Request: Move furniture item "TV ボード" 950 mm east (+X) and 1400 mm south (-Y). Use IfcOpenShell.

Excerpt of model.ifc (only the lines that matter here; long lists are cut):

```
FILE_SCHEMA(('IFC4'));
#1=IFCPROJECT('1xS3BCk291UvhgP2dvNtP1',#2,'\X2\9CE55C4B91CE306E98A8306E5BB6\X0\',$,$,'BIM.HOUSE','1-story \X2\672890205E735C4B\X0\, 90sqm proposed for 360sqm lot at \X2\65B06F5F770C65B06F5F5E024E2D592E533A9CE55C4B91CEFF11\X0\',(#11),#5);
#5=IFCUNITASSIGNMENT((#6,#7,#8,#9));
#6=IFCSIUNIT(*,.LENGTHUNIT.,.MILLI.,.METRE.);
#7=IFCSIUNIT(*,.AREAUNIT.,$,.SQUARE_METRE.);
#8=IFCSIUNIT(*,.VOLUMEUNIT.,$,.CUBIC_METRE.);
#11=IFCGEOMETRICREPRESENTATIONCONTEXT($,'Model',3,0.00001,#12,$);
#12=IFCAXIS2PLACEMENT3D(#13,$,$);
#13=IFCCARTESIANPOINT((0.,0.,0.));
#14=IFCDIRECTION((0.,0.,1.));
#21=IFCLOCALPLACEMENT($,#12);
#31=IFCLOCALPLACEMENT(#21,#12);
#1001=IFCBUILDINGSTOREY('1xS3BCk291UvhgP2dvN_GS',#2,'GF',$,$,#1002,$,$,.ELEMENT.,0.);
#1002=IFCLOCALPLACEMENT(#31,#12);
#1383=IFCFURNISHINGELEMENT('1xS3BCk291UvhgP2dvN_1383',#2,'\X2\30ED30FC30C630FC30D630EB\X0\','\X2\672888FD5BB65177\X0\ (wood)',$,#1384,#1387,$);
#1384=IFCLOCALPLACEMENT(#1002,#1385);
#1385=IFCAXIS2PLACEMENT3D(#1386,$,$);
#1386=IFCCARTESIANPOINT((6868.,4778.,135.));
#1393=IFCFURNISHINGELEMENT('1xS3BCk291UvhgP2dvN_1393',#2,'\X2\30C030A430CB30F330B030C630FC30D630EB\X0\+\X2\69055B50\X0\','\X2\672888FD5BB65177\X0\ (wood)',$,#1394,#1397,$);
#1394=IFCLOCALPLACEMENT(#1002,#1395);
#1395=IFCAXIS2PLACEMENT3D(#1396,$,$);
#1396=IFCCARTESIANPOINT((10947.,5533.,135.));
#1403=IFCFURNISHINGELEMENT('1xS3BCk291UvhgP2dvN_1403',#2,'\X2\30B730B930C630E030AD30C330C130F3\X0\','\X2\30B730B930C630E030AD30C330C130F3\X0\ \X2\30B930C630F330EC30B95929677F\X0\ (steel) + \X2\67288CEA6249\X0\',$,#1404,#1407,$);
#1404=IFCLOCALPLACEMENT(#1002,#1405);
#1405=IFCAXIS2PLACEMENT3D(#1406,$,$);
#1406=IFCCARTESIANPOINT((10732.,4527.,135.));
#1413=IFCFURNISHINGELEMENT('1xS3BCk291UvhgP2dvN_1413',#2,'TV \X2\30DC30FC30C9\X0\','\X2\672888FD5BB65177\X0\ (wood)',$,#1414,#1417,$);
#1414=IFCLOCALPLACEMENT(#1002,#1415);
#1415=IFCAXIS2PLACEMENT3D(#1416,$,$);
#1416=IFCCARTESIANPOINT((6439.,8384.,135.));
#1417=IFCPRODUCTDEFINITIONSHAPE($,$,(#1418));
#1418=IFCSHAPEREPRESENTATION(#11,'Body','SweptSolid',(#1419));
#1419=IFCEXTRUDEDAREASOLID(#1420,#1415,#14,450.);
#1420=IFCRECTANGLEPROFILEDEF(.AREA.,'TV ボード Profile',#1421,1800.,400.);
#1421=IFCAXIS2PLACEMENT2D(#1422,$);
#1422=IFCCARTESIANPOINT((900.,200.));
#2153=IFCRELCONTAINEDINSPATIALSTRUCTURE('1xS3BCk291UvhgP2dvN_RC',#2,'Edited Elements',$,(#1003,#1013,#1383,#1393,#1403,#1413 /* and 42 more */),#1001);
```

```python
import ifcopenshell
import ifcopenshell.api.geometry
import ifcopenshell.util.placement

model = ifcopenshell.open("model.ifc")

item = model.by_guid("1xS3BCk291UvhgP2dvN_1413")
matrix = ifcopenshell.util.placement.get_local_placement(item.ObjectPlacement)
matrix[0, 3] += 950.0
matrix[1, 3] -= 1400.0
ifcopenshell.api.geometry.edit_object_placement(model, product=item, matrix=matrix, is_si=False)

print(ifcopenshell.util.placement.get_local_placement(item.ObjectPlacement).round(3) + 0.0)

model.write("model_updated.ifc")
```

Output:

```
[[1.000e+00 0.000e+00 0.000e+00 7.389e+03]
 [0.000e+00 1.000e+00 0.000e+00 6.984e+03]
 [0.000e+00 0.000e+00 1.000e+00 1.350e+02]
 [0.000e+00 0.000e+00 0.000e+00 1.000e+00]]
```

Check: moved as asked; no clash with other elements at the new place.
